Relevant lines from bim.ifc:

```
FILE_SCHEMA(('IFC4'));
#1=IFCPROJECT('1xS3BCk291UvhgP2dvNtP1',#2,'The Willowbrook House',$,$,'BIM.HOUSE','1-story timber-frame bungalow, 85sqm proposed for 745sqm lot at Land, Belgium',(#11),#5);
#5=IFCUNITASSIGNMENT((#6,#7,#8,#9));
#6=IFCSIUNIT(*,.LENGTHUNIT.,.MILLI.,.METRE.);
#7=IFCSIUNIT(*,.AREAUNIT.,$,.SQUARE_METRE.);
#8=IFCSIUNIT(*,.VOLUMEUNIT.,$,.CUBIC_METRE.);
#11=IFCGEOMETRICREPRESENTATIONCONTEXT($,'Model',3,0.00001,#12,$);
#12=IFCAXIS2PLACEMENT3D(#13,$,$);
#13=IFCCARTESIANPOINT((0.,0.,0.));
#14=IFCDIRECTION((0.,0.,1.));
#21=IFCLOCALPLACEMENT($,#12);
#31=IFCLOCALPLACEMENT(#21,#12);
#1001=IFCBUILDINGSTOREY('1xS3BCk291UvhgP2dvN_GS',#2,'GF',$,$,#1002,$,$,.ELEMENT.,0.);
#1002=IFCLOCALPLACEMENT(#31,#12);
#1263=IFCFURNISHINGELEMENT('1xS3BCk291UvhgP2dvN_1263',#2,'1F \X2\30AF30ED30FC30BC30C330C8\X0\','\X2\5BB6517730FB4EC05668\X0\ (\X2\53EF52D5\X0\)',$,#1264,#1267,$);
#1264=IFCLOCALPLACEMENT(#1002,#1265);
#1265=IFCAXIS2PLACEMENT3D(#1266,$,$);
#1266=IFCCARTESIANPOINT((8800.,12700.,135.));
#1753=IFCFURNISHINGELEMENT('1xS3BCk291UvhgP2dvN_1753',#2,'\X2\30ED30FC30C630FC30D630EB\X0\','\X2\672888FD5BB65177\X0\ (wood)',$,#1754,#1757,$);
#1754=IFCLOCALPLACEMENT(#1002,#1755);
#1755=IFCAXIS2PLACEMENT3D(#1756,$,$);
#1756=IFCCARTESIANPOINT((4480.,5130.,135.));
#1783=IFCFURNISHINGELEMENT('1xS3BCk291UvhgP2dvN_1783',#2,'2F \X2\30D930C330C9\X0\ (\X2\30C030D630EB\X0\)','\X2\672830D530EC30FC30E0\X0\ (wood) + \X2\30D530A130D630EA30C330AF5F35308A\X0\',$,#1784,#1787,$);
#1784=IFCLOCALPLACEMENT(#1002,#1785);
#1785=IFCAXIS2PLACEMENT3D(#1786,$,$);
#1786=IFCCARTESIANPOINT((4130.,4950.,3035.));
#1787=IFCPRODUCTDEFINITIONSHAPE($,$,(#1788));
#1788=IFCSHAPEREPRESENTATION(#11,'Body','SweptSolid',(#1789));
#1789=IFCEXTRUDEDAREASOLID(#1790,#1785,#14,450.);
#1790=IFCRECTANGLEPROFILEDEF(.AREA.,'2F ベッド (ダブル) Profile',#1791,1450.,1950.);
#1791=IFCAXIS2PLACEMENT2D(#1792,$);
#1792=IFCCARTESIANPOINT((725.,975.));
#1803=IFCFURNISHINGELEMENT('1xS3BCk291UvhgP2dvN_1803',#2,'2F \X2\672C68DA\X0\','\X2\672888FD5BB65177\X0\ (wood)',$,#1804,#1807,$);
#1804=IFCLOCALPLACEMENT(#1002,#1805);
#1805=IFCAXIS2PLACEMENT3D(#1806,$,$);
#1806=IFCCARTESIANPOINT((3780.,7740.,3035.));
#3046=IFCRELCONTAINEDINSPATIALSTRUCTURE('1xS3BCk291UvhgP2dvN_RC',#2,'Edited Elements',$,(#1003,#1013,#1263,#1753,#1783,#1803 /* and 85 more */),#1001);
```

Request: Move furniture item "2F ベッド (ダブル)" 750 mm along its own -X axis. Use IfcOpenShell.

```python
import ifcopenshell
import ifcopenshell.api.geometry
import ifcopenshell.util.placement

model = ifcopenshell.open("bim.ifc")

item = model.by_guid("1xS3BCk291UvhgP2dvN_1783")
matrix = ifcopenshell.util.placement.get_local_placement(item.ObjectPlacement)
matrix[:3, 3] -= matrix[:3, 0] * 750.0
ifcopenshell.api.geometry.edit_object_placement(model, product=item, matrix=matrix, is_si=False)

print(ifcopenshell.util.placement.get_local_placement(item.ObjectPlacement).round(3) + 0.0)

model.write("bim_v2.ifc")
```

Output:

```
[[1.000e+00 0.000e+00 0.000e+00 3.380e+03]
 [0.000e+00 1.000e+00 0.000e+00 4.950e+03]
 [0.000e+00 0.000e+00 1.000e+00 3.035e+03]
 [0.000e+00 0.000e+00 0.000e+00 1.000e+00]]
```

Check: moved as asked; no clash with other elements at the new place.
